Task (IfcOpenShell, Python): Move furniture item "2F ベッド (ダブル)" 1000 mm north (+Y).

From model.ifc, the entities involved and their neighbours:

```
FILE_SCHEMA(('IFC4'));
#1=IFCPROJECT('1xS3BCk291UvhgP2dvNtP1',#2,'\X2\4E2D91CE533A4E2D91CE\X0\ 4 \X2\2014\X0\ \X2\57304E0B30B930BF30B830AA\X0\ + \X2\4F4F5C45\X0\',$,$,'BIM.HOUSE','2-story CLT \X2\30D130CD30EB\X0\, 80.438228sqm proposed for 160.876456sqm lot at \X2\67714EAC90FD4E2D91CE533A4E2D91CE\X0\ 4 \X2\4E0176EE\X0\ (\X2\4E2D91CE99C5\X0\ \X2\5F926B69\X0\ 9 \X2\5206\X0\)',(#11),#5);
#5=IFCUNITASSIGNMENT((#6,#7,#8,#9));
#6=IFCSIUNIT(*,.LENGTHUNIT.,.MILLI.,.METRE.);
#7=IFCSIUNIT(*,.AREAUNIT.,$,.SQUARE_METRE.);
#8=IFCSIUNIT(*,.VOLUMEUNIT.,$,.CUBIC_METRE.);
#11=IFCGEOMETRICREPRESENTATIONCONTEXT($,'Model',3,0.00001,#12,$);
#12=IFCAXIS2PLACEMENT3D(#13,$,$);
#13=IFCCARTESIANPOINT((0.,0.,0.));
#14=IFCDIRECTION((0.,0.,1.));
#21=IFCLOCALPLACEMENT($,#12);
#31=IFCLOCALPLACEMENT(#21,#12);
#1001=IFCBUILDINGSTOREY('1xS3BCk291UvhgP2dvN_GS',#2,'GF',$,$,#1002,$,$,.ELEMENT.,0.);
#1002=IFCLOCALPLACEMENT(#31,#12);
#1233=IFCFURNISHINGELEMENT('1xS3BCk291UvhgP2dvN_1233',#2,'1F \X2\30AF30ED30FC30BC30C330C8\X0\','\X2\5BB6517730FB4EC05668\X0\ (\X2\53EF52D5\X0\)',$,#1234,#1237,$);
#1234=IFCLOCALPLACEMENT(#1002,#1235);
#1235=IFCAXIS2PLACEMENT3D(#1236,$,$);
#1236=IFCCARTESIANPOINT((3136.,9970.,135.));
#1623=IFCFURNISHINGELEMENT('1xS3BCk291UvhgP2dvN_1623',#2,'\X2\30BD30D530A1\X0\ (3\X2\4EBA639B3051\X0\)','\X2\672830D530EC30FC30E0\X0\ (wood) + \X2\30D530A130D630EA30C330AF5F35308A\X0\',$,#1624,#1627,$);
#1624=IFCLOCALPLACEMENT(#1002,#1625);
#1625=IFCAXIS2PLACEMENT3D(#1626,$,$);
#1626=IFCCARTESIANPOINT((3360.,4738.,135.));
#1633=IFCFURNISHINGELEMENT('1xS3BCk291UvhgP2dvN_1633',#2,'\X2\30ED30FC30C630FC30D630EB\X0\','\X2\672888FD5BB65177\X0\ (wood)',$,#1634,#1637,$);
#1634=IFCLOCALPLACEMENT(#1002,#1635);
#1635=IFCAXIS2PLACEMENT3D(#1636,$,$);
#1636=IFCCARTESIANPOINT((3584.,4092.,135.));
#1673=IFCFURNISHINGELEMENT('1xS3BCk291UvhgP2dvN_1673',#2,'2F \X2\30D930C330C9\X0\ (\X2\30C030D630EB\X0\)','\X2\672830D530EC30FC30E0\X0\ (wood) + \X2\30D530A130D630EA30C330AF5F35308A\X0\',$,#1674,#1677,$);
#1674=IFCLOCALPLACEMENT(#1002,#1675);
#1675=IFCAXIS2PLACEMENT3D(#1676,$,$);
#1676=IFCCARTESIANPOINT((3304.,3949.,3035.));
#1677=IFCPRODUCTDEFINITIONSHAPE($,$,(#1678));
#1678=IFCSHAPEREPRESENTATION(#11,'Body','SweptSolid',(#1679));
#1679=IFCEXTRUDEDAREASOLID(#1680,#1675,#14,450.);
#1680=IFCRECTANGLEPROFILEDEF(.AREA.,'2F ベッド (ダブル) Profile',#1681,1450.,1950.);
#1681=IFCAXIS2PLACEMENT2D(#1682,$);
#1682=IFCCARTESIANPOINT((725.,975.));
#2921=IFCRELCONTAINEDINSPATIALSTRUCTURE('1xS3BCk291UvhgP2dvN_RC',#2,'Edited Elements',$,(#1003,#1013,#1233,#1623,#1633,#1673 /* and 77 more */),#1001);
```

```python
import ifcopenshell
import ifcopenshell.api.geometry
import ifcopenshell.util.placement

model = ifcopenshell.open("model.ifc")

item = model.by_guid("1xS3BCk291UvhgP2dvN_1673")
matrix = ifcopenshell.util.placement.get_local_placement(item.ObjectPlacement)
matrix[1, 3] += 1000.0
ifcopenshell.api.geometry.edit_object_placement(model, product=item, matrix=matrix, is_si=False)

print(ifcopenshell.util.placement.get_local_placement(item.ObjectPlacement).round(3) + 0.0)

model.write("model_v2.ifc")
```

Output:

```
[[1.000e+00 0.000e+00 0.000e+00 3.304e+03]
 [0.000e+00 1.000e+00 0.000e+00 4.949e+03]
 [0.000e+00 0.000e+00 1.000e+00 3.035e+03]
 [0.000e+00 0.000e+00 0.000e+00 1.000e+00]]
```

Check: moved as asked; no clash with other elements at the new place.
